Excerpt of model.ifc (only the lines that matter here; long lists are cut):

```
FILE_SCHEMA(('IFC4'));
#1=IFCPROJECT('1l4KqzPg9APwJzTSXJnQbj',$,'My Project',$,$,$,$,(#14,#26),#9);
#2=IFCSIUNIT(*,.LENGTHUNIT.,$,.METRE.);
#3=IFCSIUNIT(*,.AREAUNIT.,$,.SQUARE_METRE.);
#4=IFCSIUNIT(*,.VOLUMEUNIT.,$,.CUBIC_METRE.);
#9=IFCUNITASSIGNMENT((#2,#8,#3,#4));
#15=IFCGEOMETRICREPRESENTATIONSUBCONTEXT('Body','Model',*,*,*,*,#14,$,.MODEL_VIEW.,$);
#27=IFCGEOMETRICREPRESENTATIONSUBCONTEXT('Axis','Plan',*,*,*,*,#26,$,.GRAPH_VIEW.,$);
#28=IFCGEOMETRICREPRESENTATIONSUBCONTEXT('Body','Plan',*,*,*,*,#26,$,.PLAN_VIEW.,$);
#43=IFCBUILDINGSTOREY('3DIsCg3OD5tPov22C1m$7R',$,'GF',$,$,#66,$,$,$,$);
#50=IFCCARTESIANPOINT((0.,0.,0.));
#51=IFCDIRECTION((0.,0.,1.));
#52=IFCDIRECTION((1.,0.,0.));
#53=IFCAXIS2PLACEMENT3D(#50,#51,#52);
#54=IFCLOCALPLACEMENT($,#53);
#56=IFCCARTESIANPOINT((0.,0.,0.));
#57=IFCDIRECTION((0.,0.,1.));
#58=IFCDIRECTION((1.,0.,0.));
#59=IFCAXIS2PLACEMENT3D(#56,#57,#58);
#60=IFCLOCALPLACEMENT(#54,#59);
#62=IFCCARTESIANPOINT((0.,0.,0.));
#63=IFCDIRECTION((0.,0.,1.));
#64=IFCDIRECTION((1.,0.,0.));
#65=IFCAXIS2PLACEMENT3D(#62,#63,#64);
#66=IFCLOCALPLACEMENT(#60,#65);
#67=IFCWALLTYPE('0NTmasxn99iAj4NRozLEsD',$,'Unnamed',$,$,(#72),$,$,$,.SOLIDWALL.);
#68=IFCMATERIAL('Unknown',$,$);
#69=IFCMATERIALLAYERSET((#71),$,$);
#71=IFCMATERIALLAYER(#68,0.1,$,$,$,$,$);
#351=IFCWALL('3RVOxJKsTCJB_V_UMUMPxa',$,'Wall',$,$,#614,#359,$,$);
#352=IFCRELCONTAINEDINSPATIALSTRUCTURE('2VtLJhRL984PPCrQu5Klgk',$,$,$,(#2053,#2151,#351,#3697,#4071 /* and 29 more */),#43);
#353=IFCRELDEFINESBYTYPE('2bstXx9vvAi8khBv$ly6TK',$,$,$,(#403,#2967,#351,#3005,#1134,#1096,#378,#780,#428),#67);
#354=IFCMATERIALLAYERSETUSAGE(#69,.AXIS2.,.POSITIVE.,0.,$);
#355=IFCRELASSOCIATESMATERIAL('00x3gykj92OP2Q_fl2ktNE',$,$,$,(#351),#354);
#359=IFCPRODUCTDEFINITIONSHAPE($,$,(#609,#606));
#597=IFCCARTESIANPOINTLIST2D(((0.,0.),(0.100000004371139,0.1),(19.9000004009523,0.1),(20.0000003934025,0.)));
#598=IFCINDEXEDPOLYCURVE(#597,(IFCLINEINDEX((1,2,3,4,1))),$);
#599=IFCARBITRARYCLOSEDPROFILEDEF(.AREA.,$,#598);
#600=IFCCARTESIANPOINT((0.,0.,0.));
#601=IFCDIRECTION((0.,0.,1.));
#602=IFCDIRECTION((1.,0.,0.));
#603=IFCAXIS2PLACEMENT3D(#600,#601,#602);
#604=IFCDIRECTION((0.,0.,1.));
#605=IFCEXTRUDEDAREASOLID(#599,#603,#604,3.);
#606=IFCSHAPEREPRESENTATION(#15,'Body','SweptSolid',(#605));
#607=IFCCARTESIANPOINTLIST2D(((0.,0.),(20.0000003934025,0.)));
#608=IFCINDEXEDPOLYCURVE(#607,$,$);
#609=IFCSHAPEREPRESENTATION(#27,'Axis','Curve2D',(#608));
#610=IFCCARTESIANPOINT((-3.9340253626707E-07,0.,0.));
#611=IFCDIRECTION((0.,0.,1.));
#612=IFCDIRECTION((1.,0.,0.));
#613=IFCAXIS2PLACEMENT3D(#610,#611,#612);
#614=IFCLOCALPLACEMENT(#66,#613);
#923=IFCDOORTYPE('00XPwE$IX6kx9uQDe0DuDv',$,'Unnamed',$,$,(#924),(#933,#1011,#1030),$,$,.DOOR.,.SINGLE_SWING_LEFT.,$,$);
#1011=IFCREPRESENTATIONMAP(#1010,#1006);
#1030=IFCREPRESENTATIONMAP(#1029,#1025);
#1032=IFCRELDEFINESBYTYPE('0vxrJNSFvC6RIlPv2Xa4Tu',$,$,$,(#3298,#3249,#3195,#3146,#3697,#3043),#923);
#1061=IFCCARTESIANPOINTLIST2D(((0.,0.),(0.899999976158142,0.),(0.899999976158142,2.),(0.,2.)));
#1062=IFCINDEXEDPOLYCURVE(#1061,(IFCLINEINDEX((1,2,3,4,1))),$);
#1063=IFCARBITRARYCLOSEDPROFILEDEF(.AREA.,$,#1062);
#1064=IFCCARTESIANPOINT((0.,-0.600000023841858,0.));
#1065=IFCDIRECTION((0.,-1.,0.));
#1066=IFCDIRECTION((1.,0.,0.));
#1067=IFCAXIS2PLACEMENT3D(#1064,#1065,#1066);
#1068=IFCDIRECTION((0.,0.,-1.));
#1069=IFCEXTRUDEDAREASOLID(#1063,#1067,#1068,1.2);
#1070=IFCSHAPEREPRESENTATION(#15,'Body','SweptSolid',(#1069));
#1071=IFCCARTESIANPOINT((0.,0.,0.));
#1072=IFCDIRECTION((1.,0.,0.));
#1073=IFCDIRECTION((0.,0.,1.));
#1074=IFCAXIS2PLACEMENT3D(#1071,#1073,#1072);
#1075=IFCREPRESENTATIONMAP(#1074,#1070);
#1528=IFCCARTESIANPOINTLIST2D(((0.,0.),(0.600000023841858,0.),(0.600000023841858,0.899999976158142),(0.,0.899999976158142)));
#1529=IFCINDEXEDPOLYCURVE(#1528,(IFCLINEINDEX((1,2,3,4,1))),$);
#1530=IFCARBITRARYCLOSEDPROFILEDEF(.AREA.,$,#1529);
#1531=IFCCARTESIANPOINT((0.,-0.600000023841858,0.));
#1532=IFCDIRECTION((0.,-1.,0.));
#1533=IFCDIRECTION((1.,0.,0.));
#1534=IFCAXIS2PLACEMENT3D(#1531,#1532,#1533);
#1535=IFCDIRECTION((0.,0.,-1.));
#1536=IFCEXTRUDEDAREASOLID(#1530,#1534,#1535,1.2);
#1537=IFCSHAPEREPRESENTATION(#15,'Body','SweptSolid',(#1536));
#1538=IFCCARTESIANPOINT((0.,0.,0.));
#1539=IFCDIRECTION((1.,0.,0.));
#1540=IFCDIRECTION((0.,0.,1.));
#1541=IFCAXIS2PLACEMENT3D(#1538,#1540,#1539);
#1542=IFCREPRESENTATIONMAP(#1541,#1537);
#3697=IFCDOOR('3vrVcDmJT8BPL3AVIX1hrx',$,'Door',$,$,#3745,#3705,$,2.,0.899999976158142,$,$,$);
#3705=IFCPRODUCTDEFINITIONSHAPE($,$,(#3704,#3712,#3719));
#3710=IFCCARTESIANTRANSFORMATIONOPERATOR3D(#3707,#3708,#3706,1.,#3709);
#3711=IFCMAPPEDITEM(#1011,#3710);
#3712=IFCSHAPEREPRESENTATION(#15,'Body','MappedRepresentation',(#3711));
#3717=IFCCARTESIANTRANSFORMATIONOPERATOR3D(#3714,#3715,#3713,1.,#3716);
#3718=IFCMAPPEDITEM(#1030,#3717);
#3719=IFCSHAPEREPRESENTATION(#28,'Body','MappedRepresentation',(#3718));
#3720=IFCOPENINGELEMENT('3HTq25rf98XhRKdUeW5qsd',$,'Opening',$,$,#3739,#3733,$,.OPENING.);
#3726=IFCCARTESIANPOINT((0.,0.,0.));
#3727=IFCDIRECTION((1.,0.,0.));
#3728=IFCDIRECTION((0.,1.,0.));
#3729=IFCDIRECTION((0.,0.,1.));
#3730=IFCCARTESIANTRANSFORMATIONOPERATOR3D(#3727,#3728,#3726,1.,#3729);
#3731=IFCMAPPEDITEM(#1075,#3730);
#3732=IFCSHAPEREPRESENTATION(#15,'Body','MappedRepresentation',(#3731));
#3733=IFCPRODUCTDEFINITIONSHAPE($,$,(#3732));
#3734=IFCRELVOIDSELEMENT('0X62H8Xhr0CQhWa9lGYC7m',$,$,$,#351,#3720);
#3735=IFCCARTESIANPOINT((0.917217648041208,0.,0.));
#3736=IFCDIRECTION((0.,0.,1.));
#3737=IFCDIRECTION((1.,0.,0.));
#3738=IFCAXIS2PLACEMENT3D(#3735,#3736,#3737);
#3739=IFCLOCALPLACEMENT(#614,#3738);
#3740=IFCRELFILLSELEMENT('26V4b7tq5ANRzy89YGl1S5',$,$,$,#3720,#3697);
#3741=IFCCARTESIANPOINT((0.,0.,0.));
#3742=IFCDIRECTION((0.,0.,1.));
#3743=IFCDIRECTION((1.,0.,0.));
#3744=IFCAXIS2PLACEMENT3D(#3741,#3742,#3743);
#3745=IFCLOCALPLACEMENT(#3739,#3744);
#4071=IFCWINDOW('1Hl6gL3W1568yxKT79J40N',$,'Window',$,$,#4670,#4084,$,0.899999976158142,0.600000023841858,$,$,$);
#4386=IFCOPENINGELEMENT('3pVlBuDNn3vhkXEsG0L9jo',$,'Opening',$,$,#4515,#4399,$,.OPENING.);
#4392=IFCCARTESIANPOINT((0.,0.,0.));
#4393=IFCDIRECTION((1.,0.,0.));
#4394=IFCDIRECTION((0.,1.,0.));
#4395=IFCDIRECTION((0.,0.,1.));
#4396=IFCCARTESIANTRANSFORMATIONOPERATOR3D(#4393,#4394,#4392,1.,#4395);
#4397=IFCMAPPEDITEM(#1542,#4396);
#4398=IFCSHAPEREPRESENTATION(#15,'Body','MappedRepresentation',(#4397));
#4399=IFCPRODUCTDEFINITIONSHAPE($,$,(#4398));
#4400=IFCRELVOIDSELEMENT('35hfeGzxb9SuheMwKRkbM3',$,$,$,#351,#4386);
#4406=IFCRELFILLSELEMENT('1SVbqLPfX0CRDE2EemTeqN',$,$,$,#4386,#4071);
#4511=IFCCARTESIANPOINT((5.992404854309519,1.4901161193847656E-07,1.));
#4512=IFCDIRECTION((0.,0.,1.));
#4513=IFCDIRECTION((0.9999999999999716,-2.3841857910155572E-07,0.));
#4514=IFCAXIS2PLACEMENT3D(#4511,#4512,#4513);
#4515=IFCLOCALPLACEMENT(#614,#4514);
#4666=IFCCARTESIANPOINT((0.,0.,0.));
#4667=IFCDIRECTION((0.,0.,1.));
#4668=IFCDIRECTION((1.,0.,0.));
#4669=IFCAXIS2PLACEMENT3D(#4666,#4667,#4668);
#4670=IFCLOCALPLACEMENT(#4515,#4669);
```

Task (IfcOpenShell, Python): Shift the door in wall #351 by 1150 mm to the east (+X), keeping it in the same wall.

```python
import ifcopenshell
import ifcopenshell.api.geometry
import ifcopenshell.util.placement
import ifcopenshell.util.unit

model = ifcopenshell.open("model.ifc")
unit_scale = ifcopenshell.util.unit.calculate_unit_scale(model)

door = model.by_id(3697)
opening = door.FillsVoids[0].RelatingOpeningElement
wall = opening.VoidsElements[0].RelatingBuildingElement

wall_matrix = ifcopenshell.util.placement.get_local_placement(wall.ObjectPlacement)
shift = wall_matrix[:3, 0] * 1.15 / unit_scale
before = ifcopenshell.util.placement.get_local_placement(door.ObjectPlacement)[:3, 3].copy()

# The door is placed relative to its opening, so it follows when the opening moves.
matrix = ifcopenshell.util.placement.get_local_placement(opening.ObjectPlacement)
matrix[:3, 3] += shift
ifcopenshell.api.geometry.edit_object_placement(
    model, product=opening, matrix=matrix, is_si=False, should_transform_children=True
)

after = ifcopenshell.util.placement.get_local_placement(door.ObjectPlacement)[:3, 3]
print("door moved by", (after - before).round(3) + 0.0)

model.write("model-out.ifc")
```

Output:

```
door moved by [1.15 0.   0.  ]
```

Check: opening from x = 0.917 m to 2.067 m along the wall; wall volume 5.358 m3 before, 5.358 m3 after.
